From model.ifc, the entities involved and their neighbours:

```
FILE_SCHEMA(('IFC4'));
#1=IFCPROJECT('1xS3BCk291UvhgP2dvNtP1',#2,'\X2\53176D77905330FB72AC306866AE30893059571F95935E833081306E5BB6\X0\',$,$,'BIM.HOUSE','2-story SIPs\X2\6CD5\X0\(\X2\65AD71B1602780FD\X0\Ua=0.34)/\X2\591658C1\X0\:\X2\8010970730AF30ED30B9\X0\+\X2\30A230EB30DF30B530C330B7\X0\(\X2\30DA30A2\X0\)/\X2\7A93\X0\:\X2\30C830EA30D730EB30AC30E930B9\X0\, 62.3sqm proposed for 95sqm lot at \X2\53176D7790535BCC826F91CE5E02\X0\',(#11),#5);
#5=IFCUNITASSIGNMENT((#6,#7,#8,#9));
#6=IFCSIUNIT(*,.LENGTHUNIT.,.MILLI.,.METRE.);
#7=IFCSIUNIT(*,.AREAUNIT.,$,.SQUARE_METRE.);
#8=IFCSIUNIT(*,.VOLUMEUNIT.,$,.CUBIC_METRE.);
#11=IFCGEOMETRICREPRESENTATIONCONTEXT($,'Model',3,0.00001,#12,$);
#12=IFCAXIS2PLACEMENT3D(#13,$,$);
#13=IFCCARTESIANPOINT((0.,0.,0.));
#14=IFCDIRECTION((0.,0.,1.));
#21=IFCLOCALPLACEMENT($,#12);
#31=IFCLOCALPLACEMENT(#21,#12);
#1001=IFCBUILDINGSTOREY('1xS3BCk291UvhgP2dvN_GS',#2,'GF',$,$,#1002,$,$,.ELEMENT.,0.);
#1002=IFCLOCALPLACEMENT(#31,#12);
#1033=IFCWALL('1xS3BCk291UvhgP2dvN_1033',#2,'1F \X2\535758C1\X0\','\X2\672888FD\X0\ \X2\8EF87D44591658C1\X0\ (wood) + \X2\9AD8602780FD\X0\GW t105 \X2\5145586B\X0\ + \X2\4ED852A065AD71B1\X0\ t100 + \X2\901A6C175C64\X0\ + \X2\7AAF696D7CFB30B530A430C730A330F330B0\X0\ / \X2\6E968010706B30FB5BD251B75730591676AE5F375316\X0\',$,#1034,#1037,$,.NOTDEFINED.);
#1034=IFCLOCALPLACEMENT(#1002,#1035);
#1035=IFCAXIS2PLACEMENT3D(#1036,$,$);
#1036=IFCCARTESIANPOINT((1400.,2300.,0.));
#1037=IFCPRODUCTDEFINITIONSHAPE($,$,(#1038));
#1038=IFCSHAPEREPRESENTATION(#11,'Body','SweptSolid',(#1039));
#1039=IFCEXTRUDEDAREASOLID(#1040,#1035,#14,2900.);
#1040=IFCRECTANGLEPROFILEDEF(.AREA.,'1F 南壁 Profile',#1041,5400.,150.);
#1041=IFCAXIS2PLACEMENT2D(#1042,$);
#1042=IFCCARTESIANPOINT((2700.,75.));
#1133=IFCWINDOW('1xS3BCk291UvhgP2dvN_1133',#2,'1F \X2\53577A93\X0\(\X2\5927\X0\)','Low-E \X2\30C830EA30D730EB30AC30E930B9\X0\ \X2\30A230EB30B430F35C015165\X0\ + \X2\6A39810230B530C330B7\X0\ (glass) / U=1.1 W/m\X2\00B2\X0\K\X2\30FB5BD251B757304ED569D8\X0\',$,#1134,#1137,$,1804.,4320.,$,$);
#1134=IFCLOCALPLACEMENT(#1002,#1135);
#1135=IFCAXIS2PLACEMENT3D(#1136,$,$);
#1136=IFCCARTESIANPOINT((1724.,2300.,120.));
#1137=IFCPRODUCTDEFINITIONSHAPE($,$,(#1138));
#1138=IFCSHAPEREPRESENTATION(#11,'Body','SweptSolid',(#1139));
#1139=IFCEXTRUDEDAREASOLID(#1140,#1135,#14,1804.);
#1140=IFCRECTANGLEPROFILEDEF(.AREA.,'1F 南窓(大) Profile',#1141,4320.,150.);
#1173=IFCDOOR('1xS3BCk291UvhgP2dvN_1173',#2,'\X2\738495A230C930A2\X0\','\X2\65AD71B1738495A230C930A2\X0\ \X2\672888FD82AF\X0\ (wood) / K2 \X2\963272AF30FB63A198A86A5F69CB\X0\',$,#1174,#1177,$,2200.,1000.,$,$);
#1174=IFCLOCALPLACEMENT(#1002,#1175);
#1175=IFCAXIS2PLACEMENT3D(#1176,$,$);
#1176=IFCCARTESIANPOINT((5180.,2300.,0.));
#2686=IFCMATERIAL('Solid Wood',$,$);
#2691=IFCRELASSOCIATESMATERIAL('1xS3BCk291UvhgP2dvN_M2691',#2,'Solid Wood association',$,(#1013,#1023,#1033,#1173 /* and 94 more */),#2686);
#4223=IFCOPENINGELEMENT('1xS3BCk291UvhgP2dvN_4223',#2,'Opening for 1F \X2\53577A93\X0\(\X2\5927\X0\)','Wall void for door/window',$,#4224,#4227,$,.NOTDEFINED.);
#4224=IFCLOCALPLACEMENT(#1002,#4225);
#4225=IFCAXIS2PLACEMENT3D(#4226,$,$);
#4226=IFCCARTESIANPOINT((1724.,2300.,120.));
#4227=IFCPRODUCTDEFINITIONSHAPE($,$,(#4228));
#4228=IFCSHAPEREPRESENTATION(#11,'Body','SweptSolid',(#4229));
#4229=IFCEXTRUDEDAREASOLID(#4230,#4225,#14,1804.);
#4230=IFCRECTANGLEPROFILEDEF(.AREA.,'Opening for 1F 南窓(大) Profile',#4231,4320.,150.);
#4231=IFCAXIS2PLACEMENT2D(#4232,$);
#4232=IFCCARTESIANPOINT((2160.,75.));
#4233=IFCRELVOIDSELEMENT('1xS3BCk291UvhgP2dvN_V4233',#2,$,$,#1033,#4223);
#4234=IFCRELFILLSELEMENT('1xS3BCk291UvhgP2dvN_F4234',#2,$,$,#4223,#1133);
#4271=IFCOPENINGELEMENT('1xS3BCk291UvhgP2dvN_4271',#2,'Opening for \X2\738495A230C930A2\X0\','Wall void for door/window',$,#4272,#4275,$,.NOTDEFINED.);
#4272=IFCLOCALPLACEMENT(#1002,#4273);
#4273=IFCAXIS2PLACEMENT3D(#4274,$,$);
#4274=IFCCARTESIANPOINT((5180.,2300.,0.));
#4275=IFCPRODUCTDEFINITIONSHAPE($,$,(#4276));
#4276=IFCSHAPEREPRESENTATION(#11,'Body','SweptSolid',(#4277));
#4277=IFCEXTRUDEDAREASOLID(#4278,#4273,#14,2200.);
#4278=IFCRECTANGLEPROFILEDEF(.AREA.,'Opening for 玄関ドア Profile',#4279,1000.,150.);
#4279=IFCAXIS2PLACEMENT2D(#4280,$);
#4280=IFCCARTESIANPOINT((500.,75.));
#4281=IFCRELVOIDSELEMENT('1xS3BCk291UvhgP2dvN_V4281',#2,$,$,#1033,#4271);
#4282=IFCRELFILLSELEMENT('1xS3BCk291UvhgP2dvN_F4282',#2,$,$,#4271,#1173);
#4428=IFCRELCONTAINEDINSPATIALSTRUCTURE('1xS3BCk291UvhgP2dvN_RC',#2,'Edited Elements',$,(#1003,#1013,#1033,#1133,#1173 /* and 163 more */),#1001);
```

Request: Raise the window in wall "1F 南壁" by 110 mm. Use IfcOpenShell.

```python
import numpy as np
import ifcopenshell
import ifcopenshell.api.geometry
import ifcopenshell.util.placement
import ifcopenshell.util.unit

model = ifcopenshell.open("model.ifc")
unit_scale = ifcopenshell.util.unit.calculate_unit_scale(model)

window = model.by_guid("1xS3BCk291UvhgP2dvN_1133")
opening = window.FillsVoids[0].RelatingOpeningElement
dz = 110.0

shift = np.array([0.0, 0.0, dz])
# The window is not placed relative to its opening, so move both.
for product in (opening, window):
    matrix = ifcopenshell.util.placement.get_local_placement(product.ObjectPlacement)
    matrix[:3, 3] += shift
    ifcopenshell.api.geometry.edit_object_placement(model, product=product, matrix=matrix, is_si=False)

print(f"moved by {dz * unit_scale:+.3f} m")

model.write("model_v2.ifc")
```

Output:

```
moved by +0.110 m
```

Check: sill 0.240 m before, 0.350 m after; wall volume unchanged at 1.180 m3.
